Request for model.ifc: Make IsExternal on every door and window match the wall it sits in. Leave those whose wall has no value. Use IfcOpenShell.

First a look at what the model holds.

```python
import ifcopenshell
import ifcopenshell.util.element

model = ifcopenshell.open("model.ifc")
print(model.schema)
seen = {}
for e in model.by_type("IfcDoor") + model.by_type("IfcWindow"):
    if not e.FillsVoids:
        continue
    host = e.FillsVoids[0].RelatingOpeningElement.VoidsElements[0].RelatingBuildingElement
    own = ifcopenshell.util.element.get_pset(e, f"Pset_{e.is_a()[3:].removesuffix('StandardCase')}Common", "IsExternal")
    wall = ifcopenshell.util.element.get_pset(host, "Pset_WallCommon", "IsExternal")
    seen[e.is_a(), own, wall] = seen.get((e.is_a(), own, wall), 0) + 1
for (cls, own, wall), count in sorted(seen.items(), key=str):
    print(count, cls, "IsExternal:", own, "| host wall:", wall)
```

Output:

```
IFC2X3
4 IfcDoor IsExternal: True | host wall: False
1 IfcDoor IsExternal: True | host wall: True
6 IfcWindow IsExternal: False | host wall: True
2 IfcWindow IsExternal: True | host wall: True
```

```python
import ifcopenshell
import ifcopenshell.api.pset
import ifcopenshell.util.element

model = ifcopenshell.open("model.ifc")

count = 0
for ifc_class, pset_name in (("IfcDoor", "Pset_DoorCommon"), ("IfcWindow", "Pset_WindowCommon")):
    for e in model.by_type(ifc_class):
        if not e.FillsVoids:
            continue
        host = e.FillsVoids[0].RelatingOpeningElement.VoidsElements[0].RelatingBuildingElement
        external = ifcopenshell.util.element.get_pset(host, "Pset_WallCommon", "IsExternal")
        if external is None or ifcopenshell.util.element.get_pset(e, pset_name, "IsExternal") == external:
            continue
        pset = ifcopenshell.api.pset.add_pset(model, product=e, name=pset_name)
        ifcopenshell.api.pset.edit_pset(model, pset=pset, properties={"IsExternal": external})
        count += 1

print(count, "updated")

model.write("model_edited.ifc")
```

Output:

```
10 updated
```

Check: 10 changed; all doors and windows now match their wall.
